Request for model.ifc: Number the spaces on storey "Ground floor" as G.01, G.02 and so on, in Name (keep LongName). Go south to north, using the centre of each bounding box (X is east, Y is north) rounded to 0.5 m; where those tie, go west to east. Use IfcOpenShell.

First a look at what the model holds.

```python
import ifcopenshell
import ifcopenshell.util.element
import ifcopenshell.util.placement

model = ifcopenshell.open("model.ifc")
print(model.schema)
storey = next(s for s in model.by_type("IfcBuildingStorey") if s.Name == "Ground floor")
spaces = [e for e in ifcopenshell.util.element.get_decomposition(storey) if e.is_a("IfcSpace")]
for e in sorted(spaces, key=lambda e: e.id()):
    origin = ifcopenshell.util.placement.get_local_placement(e.ObjectPlacement)[:3, 3]
    print(e.id(), e.Name, e.LongName, origin.round(2) + 0.0, sep=" | ")
```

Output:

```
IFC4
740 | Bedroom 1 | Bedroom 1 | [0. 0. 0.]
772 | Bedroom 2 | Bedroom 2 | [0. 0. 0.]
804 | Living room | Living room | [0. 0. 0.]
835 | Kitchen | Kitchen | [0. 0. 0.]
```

```python
import ifcopenshell
import ifcopenshell.geom
import ifcopenshell.util.element
import ifcopenshell.util.shape

model = ifcopenshell.open("model.ifc")
settings = ifcopenshell.geom.settings()
settings.set("use-world-coords", True)


def centre(element):
    shape = ifcopenshell.geom.create_shape(settings, element)
    return ifcopenshell.util.shape.get_bbox_centroid(shape.geometry)


storey = next(s for s in model.by_type("IfcBuildingStorey") if s.Name == "Ground floor")
spaces = [e for e in ifcopenshell.util.element.get_decomposition(storey) if e.is_a("IfcSpace")]

# Insertion points can sit at a corner or the storey origin, so sort by the geometry (in metres).
centres = {e: centre(e) for e in spaces}
spaces.sort(key=lambda e: (round(centres[e][1] / 0.5), centres[e][0]))

for i, e in enumerate(spaces, start=1):
    number = f"G.{i:02d}"
    e.Name = number
    print(e.id(), number)

model.write("model_v2.ifc")
```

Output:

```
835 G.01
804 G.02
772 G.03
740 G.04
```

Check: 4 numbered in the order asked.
